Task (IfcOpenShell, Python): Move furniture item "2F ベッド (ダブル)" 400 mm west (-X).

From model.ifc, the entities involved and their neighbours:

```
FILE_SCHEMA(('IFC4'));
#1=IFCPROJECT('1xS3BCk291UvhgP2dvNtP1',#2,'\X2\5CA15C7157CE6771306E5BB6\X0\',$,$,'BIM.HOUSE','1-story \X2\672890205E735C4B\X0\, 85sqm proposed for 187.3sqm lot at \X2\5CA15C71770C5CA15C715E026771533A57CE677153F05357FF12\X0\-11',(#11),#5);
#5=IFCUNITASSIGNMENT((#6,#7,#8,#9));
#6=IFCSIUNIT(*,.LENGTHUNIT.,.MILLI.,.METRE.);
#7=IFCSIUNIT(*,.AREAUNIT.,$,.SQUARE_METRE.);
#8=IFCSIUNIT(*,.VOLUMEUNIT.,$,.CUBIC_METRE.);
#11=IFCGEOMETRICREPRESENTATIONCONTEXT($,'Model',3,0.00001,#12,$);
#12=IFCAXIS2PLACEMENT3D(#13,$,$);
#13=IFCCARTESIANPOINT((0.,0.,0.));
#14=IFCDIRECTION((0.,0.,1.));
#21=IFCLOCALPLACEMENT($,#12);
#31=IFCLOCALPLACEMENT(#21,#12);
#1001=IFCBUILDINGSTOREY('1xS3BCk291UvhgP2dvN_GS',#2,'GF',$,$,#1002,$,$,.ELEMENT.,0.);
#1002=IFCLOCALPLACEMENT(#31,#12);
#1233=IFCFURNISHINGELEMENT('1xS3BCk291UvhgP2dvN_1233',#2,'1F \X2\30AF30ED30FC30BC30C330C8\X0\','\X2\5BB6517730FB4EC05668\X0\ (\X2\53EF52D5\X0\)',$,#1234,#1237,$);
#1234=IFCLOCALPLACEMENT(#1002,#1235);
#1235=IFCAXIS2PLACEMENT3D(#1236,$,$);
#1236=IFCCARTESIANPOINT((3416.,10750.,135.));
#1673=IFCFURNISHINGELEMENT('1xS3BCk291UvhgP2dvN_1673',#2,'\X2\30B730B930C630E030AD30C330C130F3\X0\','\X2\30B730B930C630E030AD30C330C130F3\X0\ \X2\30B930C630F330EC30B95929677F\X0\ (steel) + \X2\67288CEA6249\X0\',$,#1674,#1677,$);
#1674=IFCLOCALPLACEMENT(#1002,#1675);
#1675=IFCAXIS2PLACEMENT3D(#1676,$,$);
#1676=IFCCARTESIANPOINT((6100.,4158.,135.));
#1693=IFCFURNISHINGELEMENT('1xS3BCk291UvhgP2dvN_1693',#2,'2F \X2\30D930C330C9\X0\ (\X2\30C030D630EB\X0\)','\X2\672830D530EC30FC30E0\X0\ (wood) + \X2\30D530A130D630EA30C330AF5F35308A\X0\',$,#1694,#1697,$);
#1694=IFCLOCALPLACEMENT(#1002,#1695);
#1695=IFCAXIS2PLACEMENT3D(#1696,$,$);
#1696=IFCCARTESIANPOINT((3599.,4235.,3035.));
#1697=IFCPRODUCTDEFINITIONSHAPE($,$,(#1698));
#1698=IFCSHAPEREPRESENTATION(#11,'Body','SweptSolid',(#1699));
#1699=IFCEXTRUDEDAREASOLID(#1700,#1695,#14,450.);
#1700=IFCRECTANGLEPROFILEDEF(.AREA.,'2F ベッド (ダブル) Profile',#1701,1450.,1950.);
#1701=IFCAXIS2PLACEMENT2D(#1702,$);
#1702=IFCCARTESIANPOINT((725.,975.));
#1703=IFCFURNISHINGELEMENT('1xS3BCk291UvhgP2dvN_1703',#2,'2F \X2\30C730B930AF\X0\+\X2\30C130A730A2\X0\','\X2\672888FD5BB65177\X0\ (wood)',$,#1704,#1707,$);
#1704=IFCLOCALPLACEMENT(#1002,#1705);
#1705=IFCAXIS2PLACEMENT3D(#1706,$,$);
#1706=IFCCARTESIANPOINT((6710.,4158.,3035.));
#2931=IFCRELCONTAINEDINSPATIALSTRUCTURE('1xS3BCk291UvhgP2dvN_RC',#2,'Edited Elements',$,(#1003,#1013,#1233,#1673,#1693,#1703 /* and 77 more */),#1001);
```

```python
import ifcopenshell
import ifcopenshell.api.geometry
import ifcopenshell.util.placement
import ifcopenshell.util.unit

model = ifcopenshell.open("model.ifc")
unit_scale = ifcopenshell.util.unit.calculate_unit_scale(model)

item = model.by_id(1693)
matrix = ifcopenshell.util.placement.get_local_placement(item.ObjectPlacement)
matrix[0, 3] -= 0.4 / unit_scale
ifcopenshell.api.geometry.edit_object_placement(model, product=item, matrix=matrix, is_si=False)

print(ifcopenshell.util.placement.get_local_placement(item.ObjectPlacement).round(3) + 0.0)

model.write("model_v2.ifc")
```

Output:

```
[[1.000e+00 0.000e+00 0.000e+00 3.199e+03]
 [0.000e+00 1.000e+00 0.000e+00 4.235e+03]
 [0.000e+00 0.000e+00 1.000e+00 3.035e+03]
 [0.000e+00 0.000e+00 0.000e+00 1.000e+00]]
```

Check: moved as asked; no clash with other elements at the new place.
